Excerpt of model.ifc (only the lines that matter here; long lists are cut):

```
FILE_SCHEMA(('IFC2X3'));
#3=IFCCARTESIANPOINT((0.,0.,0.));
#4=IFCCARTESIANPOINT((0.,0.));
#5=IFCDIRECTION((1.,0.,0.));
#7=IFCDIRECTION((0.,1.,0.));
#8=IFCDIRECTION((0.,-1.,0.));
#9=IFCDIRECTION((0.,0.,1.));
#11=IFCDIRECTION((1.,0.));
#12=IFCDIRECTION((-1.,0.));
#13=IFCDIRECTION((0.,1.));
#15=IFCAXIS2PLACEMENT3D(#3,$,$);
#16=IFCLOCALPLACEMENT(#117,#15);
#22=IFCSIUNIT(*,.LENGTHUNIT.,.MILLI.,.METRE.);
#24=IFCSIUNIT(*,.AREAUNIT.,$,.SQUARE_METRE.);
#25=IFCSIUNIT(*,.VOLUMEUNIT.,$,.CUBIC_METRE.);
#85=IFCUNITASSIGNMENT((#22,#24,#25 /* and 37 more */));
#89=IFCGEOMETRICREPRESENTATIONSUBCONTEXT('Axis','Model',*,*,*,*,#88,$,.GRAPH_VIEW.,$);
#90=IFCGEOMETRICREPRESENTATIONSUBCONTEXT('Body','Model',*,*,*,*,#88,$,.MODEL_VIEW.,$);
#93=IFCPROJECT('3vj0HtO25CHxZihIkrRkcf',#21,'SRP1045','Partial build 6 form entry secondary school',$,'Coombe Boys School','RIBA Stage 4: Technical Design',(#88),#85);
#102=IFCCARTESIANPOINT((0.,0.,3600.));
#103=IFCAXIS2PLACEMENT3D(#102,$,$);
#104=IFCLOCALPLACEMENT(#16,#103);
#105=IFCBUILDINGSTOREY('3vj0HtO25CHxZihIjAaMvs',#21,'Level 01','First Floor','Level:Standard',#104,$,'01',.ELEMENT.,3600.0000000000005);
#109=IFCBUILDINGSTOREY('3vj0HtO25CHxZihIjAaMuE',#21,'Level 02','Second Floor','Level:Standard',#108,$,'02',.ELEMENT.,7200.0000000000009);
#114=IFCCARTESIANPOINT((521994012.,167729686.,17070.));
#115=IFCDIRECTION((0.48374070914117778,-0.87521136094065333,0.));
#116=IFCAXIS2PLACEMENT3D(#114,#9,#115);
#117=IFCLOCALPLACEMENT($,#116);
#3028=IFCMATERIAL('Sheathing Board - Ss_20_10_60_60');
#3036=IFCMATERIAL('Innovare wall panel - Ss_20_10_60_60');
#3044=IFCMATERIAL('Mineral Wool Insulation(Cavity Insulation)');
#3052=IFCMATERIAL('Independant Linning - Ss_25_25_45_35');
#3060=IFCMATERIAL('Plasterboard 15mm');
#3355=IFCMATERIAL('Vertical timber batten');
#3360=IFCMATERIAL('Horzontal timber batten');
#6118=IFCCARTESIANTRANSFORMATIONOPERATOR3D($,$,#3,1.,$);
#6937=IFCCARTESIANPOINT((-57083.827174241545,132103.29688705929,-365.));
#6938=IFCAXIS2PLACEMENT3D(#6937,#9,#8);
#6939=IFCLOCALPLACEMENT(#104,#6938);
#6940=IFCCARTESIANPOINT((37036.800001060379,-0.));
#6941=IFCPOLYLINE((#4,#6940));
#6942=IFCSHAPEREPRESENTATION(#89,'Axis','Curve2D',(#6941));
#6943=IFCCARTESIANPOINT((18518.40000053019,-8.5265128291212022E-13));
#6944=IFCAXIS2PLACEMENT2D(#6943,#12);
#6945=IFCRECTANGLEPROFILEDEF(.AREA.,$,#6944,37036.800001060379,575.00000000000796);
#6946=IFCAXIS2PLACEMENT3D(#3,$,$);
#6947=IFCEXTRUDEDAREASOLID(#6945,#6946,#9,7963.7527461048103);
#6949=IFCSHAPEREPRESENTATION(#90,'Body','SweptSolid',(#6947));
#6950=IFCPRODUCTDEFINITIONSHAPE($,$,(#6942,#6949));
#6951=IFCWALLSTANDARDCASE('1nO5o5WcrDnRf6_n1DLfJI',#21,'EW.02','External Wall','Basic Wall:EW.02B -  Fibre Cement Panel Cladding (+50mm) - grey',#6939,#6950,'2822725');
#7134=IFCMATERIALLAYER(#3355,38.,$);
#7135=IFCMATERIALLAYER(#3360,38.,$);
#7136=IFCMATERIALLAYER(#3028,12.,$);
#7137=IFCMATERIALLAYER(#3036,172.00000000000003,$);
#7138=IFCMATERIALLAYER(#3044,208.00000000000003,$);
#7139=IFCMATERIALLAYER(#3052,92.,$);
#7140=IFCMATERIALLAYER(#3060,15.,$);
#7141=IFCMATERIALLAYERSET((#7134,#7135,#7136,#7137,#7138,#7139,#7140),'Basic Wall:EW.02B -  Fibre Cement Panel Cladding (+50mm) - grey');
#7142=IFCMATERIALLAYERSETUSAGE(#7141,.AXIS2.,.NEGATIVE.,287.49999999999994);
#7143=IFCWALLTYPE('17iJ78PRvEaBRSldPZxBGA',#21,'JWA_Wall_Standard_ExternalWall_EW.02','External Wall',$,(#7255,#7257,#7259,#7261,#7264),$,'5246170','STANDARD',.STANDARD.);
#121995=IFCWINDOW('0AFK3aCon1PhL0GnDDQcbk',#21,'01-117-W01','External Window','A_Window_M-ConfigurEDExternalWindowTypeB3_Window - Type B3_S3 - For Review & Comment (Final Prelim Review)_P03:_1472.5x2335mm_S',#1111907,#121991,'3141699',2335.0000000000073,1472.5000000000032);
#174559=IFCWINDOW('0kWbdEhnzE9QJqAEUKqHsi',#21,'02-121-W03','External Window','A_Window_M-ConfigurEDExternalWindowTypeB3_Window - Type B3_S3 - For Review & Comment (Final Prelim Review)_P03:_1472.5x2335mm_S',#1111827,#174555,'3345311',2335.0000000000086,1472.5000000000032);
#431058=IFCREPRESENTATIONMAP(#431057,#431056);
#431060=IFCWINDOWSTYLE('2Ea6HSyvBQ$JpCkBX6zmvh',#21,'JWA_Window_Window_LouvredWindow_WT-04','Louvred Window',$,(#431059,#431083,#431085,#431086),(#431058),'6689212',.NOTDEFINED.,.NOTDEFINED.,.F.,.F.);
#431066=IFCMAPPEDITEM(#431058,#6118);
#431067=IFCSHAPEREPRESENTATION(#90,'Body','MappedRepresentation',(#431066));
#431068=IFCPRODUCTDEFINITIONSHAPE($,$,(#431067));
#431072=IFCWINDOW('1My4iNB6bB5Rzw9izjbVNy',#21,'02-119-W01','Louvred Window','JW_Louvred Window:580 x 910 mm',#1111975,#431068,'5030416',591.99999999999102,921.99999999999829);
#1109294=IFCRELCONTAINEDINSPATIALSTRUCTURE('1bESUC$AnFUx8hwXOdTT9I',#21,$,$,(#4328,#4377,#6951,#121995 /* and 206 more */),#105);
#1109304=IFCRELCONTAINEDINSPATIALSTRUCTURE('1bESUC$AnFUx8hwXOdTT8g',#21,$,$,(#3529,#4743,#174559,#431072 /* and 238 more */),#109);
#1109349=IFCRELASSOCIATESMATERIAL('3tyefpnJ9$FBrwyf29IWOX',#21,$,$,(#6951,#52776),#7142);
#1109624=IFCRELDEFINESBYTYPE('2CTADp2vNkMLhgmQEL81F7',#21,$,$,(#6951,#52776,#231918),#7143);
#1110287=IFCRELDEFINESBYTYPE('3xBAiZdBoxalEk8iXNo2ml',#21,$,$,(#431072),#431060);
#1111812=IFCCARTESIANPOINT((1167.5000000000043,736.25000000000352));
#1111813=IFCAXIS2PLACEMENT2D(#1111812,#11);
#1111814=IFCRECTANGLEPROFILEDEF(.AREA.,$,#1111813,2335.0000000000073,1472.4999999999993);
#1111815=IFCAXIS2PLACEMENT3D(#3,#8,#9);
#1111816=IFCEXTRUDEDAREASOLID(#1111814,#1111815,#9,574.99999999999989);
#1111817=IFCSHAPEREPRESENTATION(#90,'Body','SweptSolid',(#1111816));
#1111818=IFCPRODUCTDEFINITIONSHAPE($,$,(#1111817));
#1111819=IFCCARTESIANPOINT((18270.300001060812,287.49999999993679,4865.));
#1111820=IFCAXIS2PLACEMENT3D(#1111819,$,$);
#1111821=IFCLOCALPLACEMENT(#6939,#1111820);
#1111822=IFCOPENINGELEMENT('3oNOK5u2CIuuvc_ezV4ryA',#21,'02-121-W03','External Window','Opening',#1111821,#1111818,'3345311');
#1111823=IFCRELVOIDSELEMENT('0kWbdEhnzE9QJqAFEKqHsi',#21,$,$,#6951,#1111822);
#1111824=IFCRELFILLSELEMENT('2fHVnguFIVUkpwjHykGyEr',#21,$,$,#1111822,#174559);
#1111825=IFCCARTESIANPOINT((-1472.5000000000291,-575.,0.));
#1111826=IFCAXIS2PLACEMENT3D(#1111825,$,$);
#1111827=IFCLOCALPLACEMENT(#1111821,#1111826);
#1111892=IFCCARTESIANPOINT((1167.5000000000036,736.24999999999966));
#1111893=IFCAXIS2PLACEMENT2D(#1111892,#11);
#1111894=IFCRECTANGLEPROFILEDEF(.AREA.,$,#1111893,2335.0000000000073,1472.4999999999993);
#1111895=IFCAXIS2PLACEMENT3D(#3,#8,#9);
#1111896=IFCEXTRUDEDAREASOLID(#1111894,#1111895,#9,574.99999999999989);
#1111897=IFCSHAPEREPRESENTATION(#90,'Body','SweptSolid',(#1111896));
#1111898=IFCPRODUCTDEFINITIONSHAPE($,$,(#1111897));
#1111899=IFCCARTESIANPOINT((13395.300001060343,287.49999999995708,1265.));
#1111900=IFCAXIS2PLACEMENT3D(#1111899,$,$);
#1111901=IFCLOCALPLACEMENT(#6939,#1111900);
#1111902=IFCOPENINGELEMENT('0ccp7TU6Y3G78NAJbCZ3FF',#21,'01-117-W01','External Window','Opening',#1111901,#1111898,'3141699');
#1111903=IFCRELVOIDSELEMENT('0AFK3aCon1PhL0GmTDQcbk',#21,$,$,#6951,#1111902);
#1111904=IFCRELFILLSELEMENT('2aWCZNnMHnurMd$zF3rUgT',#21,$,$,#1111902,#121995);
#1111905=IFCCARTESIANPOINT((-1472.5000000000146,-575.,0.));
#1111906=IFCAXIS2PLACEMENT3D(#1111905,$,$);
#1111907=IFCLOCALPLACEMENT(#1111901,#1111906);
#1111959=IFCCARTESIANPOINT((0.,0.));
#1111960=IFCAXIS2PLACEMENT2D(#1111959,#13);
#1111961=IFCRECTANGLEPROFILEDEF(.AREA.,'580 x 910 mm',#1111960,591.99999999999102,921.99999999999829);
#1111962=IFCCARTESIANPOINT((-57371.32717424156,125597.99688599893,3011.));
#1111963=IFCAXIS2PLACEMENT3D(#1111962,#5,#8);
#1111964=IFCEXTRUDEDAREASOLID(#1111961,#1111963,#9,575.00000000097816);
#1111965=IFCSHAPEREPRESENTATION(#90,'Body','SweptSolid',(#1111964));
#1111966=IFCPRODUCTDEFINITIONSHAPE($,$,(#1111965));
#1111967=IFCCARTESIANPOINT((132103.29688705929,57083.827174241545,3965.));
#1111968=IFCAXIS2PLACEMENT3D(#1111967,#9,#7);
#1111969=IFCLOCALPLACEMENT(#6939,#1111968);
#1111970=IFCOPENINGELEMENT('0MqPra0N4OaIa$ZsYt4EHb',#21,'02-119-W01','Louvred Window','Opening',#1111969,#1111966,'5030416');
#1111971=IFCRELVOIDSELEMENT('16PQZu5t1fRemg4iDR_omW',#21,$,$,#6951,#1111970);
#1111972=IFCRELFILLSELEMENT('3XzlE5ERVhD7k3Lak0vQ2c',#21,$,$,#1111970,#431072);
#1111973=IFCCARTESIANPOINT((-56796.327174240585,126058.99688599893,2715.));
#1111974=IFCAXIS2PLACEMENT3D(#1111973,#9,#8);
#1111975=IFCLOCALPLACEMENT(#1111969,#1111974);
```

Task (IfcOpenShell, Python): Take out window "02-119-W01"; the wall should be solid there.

```python
import ifcopenshell
import ifcopenshell.api.feature
import ifcopenshell.api.root
import ifcopenshell.geom
import ifcopenshell.util.shape

model = ifcopenshell.open("model.ifc")
settings = ifcopenshell.geom.settings()


def volume(element):
    """Net volume in cubic metres, openings subtracted."""
    shape = ifcopenshell.geom.create_shape(settings, element)
    return ifcopenshell.util.shape.get_volume(shape.geometry)


window = model.by_guid("1My4iNB6bB5Rzw9izjbVNy")
opening = window.FillsVoids[0].RelatingOpeningElement
wall = opening.VoidsElements[0].RelatingBuildingElement
before = volume(wall)

ifcopenshell.api.root.remove_product(model, product=window)
ifcopenshell.api.feature.remove_feature(model, feature=opening)

after = volume(wall)

print(f"wall volume {before:.3f} -> {after:.3f} m3")

model.write("model_updated.ifc")
```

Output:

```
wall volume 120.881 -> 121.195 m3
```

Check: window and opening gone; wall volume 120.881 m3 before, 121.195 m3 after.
